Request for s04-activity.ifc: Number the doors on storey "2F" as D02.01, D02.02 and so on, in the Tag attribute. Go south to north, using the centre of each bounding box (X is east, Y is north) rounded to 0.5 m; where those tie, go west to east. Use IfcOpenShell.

First a look at what the model holds.

```python
import ifcopenshell
import ifcopenshell.util.element
import ifcopenshell.util.placement

model = ifcopenshell.open("s04-activity.ifc")
print(model.schema)
storey = next(s for s in model.by_type("IfcBuildingStorey") if s.Name == "2F")
doors = [e for e in ifcopenshell.util.element.get_decomposition(storey) if e.is_a("IfcDoor")]
for e in sorted(doors, key=lambda e: e.id()):
    origin = ifcopenshell.util.placement.get_local_placement(e.ObjectPlacement)[:3, 3]
    print(e.id(), e.Tag, e.Name, origin.round(2) + 0.0, sep=" | ")
```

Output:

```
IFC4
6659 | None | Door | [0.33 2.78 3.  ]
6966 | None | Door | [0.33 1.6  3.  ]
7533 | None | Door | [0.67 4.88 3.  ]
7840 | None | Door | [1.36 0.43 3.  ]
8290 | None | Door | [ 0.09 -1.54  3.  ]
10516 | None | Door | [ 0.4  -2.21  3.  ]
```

```python
import ifcopenshell
import ifcopenshell.geom
import ifcopenshell.util.element
import ifcopenshell.util.shape

model = ifcopenshell.open("s04-activity.ifc")
settings = ifcopenshell.geom.settings()
settings.set("use-world-coords", True)


def centre(element):
    shape = ifcopenshell.geom.create_shape(settings, element)
    return ifcopenshell.util.shape.get_bbox_centroid(shape.geometry)


storey = next(s for s in model.by_type("IfcBuildingStorey") if s.Name == "2F")
doors = [e for e in ifcopenshell.util.element.get_decomposition(storey) if e.is_a("IfcDoor")]

# Insertion points can sit at a corner or the storey origin, so sort by the geometry (in metres).
centres = {e: centre(e) for e in doors}
doors.sort(key=lambda e: (round(centres[e][1] / 0.5), centres[e][0]))

for i, e in enumerate(doors, start=1):
    number = f"D02.{i:02d}"
    e.Tag = number
    print(e.id(), number)

model.write("s04-activity_rev.ifc")
```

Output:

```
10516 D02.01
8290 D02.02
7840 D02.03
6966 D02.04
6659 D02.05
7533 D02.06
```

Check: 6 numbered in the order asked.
